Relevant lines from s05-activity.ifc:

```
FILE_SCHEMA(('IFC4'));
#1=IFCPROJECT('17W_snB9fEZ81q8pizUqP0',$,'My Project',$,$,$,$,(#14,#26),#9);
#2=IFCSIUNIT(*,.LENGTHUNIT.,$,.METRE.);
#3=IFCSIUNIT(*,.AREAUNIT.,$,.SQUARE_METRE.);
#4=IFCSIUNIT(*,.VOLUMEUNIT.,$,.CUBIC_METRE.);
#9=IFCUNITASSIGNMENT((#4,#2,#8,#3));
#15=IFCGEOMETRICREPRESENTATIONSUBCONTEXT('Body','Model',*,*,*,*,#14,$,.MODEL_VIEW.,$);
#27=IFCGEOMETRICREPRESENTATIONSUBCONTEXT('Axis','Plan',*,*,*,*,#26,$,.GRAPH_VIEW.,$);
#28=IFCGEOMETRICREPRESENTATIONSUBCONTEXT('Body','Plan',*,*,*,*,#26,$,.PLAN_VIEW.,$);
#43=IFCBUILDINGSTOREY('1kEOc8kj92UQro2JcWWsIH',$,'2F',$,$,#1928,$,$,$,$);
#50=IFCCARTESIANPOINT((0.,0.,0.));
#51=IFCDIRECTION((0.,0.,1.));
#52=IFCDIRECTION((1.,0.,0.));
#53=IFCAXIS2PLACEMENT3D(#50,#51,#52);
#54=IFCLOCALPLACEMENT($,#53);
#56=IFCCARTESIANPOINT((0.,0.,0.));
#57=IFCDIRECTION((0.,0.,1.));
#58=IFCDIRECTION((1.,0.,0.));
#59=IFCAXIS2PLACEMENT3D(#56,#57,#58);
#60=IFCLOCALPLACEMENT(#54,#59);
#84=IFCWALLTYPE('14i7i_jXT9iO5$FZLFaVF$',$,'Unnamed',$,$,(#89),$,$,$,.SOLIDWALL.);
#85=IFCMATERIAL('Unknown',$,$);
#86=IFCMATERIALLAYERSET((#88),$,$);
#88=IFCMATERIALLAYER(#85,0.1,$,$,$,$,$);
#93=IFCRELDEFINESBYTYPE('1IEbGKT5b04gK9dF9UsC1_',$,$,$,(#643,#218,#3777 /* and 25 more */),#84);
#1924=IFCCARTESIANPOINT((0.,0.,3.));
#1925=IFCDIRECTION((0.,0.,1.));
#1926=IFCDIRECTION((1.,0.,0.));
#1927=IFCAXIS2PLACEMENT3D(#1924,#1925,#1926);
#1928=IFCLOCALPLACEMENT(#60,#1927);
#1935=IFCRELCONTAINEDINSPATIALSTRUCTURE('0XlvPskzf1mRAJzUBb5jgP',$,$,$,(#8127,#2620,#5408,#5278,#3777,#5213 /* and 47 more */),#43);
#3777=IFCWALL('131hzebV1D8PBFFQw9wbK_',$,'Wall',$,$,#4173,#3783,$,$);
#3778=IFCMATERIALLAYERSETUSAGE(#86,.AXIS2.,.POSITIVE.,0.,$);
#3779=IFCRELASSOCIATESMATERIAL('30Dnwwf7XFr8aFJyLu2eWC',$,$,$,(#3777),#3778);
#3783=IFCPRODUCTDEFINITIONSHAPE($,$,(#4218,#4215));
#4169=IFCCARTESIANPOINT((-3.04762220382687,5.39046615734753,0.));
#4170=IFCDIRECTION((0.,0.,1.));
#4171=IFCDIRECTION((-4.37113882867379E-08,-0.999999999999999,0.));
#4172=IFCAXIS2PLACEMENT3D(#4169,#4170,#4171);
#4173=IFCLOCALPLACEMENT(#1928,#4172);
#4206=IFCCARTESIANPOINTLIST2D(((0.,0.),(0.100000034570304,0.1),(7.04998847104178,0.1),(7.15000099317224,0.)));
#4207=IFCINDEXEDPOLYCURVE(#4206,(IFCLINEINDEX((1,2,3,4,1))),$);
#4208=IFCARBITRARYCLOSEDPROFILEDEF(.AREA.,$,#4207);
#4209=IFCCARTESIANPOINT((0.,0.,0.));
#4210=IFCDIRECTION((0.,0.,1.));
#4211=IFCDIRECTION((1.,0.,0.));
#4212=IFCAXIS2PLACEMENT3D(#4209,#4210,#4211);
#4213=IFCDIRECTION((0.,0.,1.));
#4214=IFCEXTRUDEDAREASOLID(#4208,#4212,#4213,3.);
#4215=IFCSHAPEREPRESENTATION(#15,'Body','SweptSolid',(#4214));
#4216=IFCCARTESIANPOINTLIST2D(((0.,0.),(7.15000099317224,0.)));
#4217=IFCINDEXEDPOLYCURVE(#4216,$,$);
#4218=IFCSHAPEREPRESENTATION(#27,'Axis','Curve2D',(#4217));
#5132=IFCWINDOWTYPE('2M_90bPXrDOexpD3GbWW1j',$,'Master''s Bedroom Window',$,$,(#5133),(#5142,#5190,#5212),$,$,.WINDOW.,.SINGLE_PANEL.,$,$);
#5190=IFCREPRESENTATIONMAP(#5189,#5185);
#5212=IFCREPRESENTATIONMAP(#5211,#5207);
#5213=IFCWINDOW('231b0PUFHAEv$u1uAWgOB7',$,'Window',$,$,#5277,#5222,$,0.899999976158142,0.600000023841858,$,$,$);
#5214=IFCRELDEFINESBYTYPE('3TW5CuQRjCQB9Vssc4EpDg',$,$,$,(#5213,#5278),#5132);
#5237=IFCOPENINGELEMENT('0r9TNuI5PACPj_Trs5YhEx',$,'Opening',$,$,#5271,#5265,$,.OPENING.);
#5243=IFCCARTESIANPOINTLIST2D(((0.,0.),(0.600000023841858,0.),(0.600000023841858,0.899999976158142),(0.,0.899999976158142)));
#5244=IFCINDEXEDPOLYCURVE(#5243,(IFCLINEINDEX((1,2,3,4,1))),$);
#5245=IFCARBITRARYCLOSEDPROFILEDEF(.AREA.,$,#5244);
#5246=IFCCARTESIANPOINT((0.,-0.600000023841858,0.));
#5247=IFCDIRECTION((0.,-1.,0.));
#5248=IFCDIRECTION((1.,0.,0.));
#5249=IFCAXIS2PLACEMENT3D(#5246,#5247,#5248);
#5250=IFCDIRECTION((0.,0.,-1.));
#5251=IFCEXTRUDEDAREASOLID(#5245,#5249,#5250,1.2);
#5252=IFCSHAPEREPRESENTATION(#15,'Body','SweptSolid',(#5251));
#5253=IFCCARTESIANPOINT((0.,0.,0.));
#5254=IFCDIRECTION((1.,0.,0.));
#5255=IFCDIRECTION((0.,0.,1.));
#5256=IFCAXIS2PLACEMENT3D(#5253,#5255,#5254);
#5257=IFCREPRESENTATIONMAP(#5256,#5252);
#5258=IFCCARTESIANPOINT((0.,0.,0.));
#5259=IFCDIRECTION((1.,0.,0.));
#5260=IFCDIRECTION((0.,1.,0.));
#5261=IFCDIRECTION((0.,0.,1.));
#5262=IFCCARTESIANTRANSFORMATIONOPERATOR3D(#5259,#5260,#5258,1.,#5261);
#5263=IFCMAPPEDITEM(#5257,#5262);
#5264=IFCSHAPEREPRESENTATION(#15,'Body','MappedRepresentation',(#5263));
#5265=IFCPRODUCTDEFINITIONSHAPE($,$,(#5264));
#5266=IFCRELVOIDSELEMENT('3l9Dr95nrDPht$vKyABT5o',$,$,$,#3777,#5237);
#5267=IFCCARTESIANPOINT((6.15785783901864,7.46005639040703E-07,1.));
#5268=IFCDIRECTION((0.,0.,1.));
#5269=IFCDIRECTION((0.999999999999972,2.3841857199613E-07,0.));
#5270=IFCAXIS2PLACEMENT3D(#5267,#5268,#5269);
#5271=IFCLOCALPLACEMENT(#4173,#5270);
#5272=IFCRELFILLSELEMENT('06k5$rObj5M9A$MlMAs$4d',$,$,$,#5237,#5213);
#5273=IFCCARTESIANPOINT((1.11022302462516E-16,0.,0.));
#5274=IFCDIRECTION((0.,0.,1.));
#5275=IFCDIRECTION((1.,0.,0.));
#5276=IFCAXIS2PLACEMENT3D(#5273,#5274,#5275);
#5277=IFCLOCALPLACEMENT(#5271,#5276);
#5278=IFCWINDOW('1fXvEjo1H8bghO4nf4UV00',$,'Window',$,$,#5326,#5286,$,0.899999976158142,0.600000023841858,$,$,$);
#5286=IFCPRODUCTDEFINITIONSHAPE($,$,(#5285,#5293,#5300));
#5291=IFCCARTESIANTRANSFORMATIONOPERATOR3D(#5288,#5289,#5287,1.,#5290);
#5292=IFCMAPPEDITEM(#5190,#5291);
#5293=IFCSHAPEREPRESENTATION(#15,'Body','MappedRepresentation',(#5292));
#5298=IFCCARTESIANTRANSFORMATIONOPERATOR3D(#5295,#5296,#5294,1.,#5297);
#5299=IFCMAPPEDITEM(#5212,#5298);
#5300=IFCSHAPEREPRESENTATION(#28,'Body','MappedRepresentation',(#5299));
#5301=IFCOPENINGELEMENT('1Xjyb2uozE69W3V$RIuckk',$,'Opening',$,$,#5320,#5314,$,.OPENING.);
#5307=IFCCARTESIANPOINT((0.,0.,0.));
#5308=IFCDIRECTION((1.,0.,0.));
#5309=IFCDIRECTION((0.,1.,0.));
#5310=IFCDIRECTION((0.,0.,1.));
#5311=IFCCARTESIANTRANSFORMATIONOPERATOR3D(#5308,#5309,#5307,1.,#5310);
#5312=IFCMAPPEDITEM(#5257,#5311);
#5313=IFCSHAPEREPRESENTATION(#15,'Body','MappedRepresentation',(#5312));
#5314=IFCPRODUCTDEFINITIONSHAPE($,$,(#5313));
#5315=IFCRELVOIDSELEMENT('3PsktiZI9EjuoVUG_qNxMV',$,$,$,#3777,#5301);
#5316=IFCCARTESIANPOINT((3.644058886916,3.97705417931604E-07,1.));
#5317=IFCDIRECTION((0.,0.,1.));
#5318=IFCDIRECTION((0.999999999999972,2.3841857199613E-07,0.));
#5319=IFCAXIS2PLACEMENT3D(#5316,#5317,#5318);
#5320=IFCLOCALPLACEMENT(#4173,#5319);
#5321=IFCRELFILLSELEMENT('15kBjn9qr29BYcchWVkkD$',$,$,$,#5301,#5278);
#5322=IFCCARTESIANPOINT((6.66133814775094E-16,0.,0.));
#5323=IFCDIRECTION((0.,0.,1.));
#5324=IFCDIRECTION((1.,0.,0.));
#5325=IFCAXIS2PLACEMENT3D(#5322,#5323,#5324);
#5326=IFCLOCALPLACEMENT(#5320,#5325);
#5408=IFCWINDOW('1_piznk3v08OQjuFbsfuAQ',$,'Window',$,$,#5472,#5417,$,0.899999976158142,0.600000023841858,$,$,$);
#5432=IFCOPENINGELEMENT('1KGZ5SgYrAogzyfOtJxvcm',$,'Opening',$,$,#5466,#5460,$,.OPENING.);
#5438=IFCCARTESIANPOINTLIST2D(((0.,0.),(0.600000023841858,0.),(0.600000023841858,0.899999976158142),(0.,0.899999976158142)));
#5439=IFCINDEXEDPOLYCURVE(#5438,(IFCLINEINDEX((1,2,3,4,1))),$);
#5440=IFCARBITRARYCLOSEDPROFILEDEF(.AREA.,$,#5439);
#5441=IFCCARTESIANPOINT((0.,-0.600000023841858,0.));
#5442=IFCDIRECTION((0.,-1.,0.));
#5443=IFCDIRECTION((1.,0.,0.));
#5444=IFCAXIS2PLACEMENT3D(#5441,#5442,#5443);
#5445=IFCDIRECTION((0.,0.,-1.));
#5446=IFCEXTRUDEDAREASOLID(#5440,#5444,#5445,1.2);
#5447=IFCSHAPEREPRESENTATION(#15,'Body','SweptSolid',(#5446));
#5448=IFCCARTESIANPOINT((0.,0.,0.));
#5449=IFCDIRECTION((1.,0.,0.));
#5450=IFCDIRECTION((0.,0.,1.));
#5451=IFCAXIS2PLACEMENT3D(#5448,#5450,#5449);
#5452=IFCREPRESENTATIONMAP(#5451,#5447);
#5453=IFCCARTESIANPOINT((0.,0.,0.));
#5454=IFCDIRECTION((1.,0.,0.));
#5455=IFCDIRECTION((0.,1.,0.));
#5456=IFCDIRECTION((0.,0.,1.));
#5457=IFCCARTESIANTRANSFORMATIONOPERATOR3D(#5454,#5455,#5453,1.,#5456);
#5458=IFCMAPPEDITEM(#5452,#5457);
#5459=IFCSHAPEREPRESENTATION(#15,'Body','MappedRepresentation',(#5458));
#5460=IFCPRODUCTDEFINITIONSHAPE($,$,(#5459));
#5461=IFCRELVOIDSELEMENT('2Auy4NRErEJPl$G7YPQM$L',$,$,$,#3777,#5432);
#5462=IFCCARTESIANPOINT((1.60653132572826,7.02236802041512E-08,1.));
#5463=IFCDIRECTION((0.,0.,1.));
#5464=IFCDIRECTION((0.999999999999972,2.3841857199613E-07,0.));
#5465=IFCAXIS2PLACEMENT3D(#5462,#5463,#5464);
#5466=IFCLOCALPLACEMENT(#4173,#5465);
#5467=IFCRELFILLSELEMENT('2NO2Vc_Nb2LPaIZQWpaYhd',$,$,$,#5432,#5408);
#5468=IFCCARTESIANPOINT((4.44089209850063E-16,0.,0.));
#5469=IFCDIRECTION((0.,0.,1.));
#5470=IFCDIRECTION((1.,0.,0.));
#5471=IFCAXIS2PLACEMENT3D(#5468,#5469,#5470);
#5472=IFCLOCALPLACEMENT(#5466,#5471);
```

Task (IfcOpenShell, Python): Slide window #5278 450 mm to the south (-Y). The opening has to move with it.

```python
import ifcopenshell
import ifcopenshell.api.geometry
import ifcopenshell.util.placement

model = ifcopenshell.open("s05-activity.ifc")

window = model.by_guid("1fXvEjo1H8bghO4nf4UV00")
opening = window.FillsVoids[0].RelatingOpeningElement
wall = opening.VoidsElements[0].RelatingBuildingElement

wall_matrix = ifcopenshell.util.placement.get_local_placement(wall.ObjectPlacement)
shift = wall_matrix[:3, 0] * 0.45
before = ifcopenshell.util.placement.get_local_placement(window.ObjectPlacement)[:3, 3].copy()

# The window is placed relative to its opening, so it follows when the opening moves.
matrix = ifcopenshell.util.placement.get_local_placement(opening.ObjectPlacement)
matrix[:3, 3] += shift
ifcopenshell.api.geometry.edit_object_placement(
    model, product=opening, matrix=matrix, is_si=False, should_transform_children=True
)

after = ifcopenshell.util.placement.get_local_placement(window.ObjectPlacement)[:3, 3]
print("window moved by", (after - before).round(3) + 0.0)

model.write("s05-activity_edited.ifc")
```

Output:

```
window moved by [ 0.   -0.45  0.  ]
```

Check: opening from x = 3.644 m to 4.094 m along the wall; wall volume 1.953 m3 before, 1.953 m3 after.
